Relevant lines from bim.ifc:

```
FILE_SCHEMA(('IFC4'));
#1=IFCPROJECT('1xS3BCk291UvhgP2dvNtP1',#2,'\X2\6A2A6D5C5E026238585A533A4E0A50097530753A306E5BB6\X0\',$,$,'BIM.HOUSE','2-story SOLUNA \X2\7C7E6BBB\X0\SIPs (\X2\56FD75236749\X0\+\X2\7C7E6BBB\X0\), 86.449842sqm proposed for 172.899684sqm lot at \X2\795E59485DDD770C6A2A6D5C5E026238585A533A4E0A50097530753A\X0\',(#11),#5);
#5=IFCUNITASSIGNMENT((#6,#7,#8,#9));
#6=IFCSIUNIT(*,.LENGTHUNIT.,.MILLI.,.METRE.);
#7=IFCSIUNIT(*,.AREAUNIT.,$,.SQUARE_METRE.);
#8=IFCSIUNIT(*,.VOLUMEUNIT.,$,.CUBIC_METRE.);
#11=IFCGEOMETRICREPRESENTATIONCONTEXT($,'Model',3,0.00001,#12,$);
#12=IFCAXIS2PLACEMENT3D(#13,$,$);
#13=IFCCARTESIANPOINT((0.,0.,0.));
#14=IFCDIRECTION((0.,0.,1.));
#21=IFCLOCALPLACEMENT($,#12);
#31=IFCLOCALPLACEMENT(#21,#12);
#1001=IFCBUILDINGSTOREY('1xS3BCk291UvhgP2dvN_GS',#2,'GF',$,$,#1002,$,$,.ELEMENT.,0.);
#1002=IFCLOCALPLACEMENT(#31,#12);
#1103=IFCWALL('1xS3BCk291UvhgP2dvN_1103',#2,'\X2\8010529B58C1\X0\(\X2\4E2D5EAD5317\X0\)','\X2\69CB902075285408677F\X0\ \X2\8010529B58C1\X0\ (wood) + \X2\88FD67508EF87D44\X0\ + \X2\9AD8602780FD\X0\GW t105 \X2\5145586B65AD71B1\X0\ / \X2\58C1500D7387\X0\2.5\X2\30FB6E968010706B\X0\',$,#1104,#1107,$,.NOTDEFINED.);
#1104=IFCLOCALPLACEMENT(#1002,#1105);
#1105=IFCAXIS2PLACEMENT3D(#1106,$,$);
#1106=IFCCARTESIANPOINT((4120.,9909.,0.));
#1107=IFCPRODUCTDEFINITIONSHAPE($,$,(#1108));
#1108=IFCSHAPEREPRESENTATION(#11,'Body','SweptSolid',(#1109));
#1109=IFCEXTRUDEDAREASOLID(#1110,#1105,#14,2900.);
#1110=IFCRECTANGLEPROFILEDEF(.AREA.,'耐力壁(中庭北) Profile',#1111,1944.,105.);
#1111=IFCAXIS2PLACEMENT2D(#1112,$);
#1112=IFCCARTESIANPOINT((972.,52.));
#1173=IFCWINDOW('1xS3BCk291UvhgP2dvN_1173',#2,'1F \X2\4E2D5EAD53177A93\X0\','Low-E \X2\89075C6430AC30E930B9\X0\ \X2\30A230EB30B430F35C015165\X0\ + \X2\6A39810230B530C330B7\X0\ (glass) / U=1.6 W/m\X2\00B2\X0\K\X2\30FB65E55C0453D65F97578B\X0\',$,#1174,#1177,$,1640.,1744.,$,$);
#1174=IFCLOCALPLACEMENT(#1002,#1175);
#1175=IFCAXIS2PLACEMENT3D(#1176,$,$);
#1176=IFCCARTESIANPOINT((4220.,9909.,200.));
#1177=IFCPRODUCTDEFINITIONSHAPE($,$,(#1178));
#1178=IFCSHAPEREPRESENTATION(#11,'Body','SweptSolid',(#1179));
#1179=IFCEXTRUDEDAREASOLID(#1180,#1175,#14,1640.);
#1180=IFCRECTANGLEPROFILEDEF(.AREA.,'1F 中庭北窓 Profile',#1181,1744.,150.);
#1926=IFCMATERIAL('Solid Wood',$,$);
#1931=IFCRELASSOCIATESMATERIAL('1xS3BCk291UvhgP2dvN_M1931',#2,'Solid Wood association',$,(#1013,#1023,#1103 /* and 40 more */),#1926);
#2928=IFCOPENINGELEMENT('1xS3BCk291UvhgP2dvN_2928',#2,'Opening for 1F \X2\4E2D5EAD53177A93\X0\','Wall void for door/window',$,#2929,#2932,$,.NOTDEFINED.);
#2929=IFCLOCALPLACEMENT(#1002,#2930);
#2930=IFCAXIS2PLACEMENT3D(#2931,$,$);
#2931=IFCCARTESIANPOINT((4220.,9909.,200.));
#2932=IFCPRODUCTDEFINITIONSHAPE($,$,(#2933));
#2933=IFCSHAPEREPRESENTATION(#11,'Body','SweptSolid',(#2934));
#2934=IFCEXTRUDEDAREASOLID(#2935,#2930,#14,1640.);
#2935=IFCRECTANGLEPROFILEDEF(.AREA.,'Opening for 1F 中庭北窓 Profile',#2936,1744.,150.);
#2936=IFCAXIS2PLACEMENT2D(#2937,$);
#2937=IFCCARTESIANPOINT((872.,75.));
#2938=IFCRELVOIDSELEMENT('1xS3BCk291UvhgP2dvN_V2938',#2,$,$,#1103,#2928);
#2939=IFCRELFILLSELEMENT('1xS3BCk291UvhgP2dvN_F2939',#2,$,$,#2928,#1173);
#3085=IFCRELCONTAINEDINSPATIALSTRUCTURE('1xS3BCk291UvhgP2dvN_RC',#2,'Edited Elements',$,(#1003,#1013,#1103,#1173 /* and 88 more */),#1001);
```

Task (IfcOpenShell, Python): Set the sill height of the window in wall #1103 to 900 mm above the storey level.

```python
import numpy as np
import ifcopenshell
import ifcopenshell.api.geometry
import ifcopenshell.geom
import ifcopenshell.util.element
import ifcopenshell.util.placement
import ifcopenshell.util.shape
import ifcopenshell.util.unit

model = ifcopenshell.open("bim.ifc")
unit_scale = ifcopenshell.util.unit.calculate_unit_scale(model)

window = model.by_guid("1xS3BCk291UvhgP2dvN_1173")
opening = window.FillsVoids[0].RelatingOpeningElement
storey = ifcopenshell.util.element.get_container(window, ifc_class="IfcBuildingStorey")
level = ifcopenshell.util.placement.get_local_placement(storey.ObjectPlacement)[2, 3]

# The opening's origin need not be at the sill, so measure its lowest point.
shape = ifcopenshell.geom.create_shape(ifcopenshell.geom.settings(), opening)
bottom = ifcopenshell.util.shape.get_shape_bottom_elevation(shape, shape.geometry) / unit_scale
dz = level + 900.0 - bottom

shift = np.array([0.0, 0.0, dz])
# The window is not placed relative to its opening, so move both.
for product in (opening, window):
    matrix = ifcopenshell.util.placement.get_local_placement(product.ObjectPlacement)
    matrix[:3, 3] += shift
    ifcopenshell.api.geometry.edit_object_placement(model, product=product, matrix=matrix, is_si=False)

print(f"moved by {dz * unit_scale:+.3f} m")

model.write("bim_updated.ifc")
```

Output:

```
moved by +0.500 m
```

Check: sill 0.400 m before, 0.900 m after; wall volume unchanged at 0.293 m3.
